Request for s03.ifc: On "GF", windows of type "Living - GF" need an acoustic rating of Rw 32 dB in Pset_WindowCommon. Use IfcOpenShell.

First a look at what the model holds.

```python
import ifcopenshell
import ifcopenshell.util.element

model = ifcopenshell.open("s03.ifc")
print(model.schema)
storey = next(s for s in model.by_type("IfcBuildingStorey") if s.Name == "GF")
windows = [e for e in ifcopenshell.util.element.get_decomposition(storey) if e.is_a("IfcWindow")]
seen = {}
for e in windows:
    element_type = ifcopenshell.util.element.get_type(e)
    key = (element_type.Name if element_type != e and element_type else None, ifcopenshell.util.element.get_pset(e, "Pset_WindowCommon", "AcousticRating"))
    seen[key] = seen.get(key, 0) + 1
for (name, value), count in sorted(seen.items(), key=str):
    print(count, "x", name, "|", value)
```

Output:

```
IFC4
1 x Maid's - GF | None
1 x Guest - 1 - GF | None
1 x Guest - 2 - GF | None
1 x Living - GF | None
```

```python
import ifcopenshell
import ifcopenshell.api.pset
import ifcopenshell.util.element

model = ifcopenshell.open("s03.ifc")

storey = next(s for s in model.by_type("IfcBuildingStorey") if s.Name == "GF")
windows = [e for e in ifcopenshell.util.element.get_decomposition(storey) if e.is_a("IfcWindow")]

count = 0
for e in windows:
    element_type = ifcopenshell.util.element.get_type(e)
    if element_type in (None, e) or element_type.Name != "Living - GF":
        continue
    # add_pset returns the element's existing set when there is one.
    pset = ifcopenshell.api.pset.add_pset(model, product=e, name="Pset_WindowCommon")
    ifcopenshell.api.pset.edit_pset(model, pset=pset, properties={"AcousticRating": "Rw 32 dB"})
    count += 1

print(count, "windows updated")

model.write("s03_v2.ifc")
```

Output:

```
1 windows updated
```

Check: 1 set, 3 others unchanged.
